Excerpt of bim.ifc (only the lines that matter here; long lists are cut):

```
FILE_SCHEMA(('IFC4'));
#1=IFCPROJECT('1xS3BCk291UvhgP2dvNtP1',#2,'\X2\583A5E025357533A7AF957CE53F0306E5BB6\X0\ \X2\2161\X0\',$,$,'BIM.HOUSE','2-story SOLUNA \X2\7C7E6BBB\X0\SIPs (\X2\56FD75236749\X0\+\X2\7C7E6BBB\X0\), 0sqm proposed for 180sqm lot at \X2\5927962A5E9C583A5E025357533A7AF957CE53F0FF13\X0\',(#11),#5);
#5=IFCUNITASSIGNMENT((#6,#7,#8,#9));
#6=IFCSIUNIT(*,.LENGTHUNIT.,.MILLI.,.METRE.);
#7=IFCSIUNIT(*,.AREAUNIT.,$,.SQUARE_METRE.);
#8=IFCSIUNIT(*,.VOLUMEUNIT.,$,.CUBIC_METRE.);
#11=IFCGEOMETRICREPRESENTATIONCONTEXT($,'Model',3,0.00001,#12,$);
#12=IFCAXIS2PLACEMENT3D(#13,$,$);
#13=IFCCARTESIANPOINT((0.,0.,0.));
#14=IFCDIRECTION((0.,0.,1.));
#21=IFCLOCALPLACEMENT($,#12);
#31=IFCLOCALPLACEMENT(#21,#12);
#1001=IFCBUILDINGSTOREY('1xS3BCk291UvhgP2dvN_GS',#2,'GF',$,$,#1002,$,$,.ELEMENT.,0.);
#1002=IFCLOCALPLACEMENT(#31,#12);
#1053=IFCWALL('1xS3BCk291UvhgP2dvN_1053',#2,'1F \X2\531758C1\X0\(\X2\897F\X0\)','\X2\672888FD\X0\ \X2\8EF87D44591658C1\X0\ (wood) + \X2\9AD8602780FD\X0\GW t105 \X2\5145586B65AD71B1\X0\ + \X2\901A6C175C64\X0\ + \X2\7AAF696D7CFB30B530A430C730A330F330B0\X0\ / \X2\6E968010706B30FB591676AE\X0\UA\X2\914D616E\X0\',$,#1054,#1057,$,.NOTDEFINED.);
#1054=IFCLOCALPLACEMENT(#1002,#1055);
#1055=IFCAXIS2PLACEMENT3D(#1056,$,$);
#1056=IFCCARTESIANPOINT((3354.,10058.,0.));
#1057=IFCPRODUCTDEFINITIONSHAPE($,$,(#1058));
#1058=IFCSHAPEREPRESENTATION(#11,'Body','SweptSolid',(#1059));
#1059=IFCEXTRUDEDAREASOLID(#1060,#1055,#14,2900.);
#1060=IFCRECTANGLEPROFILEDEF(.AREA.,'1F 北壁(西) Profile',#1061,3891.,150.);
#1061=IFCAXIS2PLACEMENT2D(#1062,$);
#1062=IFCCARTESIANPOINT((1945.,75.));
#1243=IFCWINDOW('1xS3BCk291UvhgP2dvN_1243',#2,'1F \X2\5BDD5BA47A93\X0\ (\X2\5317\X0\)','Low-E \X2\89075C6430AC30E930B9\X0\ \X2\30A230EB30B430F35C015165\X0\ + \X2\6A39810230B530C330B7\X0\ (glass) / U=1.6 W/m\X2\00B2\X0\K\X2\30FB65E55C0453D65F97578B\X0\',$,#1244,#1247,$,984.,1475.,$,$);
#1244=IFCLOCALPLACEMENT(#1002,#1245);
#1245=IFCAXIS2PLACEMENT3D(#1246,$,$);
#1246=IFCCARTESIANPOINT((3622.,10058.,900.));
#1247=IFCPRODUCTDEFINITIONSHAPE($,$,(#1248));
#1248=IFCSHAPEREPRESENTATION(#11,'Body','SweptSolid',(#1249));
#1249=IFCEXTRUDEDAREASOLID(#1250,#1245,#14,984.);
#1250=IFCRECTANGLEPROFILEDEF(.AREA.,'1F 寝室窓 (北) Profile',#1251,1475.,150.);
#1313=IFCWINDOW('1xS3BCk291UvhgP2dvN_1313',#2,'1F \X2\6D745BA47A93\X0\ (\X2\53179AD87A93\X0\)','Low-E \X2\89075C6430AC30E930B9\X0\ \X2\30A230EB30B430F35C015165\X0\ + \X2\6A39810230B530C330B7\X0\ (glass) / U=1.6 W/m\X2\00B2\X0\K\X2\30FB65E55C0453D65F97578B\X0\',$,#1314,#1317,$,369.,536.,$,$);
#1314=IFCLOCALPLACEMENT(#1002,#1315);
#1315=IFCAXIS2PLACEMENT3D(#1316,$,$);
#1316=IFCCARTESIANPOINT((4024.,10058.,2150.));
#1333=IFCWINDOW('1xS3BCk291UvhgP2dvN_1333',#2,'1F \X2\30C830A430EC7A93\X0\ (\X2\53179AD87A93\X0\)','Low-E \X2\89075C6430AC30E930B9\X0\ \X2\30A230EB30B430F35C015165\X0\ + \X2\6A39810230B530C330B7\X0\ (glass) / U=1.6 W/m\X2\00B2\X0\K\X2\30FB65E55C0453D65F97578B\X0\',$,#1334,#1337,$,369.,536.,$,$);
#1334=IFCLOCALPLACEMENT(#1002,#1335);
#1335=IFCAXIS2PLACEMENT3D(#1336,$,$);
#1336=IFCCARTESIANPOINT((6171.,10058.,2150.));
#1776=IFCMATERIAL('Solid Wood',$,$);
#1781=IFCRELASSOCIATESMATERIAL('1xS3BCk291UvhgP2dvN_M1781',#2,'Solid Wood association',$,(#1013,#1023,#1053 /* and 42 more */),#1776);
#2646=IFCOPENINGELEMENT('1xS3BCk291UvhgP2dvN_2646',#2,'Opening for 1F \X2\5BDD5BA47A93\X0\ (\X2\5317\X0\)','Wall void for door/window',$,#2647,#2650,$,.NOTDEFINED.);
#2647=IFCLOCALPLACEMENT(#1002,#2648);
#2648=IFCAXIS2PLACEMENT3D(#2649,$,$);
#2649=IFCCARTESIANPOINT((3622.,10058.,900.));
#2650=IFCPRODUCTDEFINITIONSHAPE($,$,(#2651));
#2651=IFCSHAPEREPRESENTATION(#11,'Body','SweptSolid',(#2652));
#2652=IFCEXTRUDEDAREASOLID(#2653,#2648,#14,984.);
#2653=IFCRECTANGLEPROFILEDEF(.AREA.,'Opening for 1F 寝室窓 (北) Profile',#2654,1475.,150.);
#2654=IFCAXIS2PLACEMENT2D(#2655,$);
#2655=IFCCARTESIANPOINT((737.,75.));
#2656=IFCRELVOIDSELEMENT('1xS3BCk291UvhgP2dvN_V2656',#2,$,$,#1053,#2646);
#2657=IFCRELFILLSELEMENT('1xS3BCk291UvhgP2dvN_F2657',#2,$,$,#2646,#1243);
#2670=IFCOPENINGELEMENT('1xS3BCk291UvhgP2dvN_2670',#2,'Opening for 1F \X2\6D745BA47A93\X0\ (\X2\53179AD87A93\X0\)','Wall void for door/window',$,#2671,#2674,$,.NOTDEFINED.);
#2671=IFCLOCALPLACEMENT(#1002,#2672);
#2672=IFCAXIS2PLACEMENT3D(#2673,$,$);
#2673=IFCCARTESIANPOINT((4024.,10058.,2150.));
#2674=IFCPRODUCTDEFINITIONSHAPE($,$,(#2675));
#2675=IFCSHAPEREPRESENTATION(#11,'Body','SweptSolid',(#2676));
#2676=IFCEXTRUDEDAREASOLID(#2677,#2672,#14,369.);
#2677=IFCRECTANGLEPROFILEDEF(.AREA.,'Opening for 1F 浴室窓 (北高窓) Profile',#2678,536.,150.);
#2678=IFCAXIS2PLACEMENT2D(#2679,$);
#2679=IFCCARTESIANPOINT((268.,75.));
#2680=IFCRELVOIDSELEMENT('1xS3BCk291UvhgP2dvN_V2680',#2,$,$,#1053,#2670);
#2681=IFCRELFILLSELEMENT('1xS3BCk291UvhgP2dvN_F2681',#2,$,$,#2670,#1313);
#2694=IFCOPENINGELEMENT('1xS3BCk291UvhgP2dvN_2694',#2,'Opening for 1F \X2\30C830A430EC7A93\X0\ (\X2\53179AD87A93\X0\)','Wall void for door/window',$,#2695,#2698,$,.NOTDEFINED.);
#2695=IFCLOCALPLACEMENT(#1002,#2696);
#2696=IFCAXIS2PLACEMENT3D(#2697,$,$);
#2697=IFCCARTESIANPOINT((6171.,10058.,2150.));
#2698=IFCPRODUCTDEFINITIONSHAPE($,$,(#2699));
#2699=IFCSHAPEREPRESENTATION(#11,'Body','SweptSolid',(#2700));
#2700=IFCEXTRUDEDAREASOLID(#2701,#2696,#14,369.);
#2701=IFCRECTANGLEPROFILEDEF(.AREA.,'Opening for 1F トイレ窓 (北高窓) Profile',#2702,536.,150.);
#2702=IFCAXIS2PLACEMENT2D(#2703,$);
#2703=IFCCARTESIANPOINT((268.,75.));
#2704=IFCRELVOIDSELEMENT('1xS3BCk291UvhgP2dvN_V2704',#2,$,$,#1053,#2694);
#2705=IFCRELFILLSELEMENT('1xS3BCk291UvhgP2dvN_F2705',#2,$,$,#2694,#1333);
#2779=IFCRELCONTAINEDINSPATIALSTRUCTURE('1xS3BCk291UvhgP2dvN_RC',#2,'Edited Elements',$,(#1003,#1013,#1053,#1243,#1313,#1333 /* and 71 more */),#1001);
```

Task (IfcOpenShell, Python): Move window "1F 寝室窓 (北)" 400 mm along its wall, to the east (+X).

```python
import ifcopenshell
import ifcopenshell.api.geometry
import ifcopenshell.util.placement

model = ifcopenshell.open("bim.ifc")

window = model.by_guid("1xS3BCk291UvhgP2dvN_1243")
opening = window.FillsVoids[0].RelatingOpeningElement
wall = opening.VoidsElements[0].RelatingBuildingElement

wall_matrix = ifcopenshell.util.placement.get_local_placement(wall.ObjectPlacement)
shift = wall_matrix[:3, 0] * 400.0
before = ifcopenshell.util.placement.get_local_placement(window.ObjectPlacement)[:3, 3].copy()

# The window is not placed relative to its opening, so move both.
for product in (opening, window):
    matrix = ifcopenshell.util.placement.get_local_placement(product.ObjectPlacement)
    matrix[:3, 3] += shift
    ifcopenshell.api.geometry.edit_object_placement(model, product=product, matrix=matrix, is_si=False)

after = ifcopenshell.util.placement.get_local_placement(window.ObjectPlacement)[:3, 3]
print("window moved by", (after - before).round(3) + 0.0)

model.write("bim_updated.ifc")
```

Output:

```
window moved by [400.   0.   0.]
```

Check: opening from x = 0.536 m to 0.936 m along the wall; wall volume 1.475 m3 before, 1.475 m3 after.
